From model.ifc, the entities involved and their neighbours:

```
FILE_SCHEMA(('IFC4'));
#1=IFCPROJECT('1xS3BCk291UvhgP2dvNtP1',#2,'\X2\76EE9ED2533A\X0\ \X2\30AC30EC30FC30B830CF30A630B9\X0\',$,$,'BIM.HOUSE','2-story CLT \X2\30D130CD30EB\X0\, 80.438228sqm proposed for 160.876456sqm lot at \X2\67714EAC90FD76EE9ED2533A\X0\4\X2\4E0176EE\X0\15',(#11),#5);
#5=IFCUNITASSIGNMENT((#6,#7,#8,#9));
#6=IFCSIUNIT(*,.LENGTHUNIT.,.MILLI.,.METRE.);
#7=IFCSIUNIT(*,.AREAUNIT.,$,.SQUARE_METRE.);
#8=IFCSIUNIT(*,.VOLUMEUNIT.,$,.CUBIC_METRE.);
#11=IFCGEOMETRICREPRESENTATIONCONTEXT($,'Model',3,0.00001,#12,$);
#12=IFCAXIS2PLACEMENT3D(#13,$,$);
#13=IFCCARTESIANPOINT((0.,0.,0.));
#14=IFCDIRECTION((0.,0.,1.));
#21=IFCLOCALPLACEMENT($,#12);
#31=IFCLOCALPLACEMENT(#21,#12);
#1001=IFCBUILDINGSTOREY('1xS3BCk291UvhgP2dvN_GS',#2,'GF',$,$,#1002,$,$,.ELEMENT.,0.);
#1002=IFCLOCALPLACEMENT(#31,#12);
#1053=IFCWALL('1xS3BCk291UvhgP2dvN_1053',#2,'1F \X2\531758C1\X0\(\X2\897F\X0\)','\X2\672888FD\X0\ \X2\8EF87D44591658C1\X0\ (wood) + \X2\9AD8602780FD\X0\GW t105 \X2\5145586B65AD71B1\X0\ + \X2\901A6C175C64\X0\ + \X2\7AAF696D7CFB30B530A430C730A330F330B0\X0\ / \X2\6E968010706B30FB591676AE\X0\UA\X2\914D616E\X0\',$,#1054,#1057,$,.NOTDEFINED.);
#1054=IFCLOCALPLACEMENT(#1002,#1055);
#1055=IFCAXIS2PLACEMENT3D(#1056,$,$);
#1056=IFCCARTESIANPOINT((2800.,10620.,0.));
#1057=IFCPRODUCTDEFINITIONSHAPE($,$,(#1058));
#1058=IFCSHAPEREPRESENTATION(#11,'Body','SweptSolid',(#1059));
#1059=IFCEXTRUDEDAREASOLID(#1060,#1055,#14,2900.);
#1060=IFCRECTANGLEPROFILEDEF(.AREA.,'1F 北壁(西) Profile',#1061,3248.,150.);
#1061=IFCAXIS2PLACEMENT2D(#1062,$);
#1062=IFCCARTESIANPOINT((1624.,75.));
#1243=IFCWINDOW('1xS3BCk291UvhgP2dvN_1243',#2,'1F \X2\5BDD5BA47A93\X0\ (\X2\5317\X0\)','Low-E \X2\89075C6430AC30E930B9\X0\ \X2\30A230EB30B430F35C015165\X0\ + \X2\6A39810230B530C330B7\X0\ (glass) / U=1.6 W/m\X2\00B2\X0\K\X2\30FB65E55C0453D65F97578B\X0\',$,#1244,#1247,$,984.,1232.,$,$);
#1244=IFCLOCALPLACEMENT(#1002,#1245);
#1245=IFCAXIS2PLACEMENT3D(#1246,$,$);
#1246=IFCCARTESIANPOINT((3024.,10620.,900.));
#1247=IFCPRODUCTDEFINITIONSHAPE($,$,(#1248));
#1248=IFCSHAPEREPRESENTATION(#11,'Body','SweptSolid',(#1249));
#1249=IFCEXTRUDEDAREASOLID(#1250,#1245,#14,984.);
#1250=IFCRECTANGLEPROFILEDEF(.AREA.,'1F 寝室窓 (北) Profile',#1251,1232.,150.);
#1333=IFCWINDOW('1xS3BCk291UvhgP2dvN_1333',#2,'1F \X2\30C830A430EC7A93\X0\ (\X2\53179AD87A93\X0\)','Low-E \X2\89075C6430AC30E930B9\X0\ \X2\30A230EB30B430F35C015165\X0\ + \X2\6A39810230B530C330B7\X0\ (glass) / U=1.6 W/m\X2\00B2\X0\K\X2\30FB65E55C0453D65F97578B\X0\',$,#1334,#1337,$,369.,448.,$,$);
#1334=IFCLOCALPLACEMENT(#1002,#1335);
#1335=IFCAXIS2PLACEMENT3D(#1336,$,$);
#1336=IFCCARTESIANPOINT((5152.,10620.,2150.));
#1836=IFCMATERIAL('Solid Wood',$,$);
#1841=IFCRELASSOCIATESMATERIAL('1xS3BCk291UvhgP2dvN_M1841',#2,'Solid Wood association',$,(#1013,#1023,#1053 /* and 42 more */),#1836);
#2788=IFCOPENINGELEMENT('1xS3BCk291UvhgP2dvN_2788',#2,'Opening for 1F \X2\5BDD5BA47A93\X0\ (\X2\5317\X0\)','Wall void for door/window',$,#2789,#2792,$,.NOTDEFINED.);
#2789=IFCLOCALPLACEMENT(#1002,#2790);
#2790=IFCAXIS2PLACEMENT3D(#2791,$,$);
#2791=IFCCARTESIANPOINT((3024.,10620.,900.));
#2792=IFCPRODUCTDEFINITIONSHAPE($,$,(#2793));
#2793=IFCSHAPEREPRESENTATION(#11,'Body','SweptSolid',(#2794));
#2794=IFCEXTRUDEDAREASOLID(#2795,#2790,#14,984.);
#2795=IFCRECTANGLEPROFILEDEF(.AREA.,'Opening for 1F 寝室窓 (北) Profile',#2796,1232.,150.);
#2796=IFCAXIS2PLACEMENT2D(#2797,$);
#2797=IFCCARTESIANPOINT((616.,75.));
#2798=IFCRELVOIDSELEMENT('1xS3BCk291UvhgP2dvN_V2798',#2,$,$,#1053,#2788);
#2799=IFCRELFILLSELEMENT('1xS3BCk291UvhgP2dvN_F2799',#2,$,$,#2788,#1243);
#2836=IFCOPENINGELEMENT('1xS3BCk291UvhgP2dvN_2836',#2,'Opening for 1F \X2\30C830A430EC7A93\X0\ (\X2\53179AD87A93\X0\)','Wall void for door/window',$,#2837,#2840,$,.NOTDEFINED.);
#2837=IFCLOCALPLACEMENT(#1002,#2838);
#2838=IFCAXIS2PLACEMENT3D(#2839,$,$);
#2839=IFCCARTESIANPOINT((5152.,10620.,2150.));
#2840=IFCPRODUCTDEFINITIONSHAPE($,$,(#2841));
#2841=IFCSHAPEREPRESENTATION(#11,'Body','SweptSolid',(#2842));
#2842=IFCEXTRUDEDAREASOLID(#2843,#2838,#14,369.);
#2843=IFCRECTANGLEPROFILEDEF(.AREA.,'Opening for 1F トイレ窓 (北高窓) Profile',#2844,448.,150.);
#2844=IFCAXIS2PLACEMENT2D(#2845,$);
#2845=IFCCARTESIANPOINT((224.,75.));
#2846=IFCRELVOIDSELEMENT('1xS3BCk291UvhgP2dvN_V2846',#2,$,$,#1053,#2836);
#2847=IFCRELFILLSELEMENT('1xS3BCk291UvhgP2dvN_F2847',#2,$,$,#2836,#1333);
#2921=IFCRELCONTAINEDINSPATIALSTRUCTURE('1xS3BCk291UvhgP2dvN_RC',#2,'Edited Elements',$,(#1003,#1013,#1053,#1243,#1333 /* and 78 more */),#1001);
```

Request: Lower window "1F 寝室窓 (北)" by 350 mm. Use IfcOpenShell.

```python
import numpy as np
import ifcopenshell
import ifcopenshell.api.geometry
import ifcopenshell.util.placement
import ifcopenshell.util.unit

model = ifcopenshell.open("model.ifc")
unit_scale = ifcopenshell.util.unit.calculate_unit_scale(model)

window = model.by_guid("1xS3BCk291UvhgP2dvN_1243")
opening = window.FillsVoids[0].RelatingOpeningElement
dz = -0.35 / unit_scale

shift = np.array([0.0, 0.0, dz])
# The window is not placed relative to its opening, so move both.
for product in (opening, window):
    matrix = ifcopenshell.util.placement.get_local_placement(product.ObjectPlacement)
    matrix[:3, 3] += shift
    ifcopenshell.api.geometry.edit_object_placement(model, product=product, matrix=matrix, is_si=False)

print(f"moved by {dz * unit_scale:+.3f} m")

model.write("model_v2.ifc")
```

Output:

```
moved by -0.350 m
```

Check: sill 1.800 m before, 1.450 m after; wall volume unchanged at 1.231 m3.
